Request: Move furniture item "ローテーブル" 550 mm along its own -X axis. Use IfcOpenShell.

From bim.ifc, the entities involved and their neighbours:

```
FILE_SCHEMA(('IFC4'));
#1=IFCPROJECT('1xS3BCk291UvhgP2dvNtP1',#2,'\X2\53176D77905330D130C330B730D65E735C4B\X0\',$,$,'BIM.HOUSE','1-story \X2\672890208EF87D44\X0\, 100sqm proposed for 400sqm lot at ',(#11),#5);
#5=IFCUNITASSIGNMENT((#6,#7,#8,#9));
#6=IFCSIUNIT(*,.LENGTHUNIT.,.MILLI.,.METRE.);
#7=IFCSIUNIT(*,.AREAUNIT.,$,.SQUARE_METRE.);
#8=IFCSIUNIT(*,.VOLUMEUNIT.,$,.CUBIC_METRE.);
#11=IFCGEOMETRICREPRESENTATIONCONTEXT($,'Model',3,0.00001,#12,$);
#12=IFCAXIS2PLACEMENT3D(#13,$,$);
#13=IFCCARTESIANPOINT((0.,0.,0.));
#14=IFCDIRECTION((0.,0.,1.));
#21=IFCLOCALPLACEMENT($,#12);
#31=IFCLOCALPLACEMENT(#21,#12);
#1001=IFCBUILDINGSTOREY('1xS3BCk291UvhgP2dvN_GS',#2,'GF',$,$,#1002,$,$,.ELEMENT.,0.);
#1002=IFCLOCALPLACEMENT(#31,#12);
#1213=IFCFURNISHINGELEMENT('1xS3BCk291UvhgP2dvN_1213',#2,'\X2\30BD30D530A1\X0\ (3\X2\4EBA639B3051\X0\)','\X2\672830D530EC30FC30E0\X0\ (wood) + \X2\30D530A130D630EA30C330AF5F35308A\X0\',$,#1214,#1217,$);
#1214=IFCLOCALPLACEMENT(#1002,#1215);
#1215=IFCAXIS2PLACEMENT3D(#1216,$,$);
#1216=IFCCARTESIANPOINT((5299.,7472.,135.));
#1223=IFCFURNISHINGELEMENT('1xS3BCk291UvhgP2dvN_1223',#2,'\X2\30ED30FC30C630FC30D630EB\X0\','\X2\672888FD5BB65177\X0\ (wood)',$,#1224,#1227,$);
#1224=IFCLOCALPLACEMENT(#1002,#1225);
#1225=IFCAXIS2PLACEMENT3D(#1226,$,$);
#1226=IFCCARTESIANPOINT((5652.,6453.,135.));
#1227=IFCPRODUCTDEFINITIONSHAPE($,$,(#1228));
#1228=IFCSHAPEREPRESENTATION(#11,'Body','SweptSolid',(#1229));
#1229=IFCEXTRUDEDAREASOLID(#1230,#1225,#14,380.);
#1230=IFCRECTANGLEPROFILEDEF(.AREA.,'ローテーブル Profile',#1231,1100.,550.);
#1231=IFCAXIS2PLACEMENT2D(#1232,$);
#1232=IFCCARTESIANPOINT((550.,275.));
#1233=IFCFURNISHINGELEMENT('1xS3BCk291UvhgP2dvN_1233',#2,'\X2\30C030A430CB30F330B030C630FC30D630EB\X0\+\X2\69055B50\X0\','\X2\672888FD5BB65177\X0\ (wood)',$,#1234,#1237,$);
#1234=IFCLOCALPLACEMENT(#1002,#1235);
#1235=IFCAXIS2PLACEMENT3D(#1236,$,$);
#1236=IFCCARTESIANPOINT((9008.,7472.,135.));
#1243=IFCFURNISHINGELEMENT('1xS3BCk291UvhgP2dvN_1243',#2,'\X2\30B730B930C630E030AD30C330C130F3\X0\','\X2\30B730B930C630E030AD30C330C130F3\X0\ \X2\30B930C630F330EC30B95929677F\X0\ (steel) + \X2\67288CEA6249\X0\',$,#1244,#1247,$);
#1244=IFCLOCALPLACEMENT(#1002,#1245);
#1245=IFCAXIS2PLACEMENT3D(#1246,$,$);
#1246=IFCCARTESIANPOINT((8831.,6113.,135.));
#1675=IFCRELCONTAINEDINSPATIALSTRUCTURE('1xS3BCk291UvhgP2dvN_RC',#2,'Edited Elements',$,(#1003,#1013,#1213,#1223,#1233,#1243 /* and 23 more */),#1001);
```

```python
import ifcopenshell
import ifcopenshell.api.geometry
import ifcopenshell.util.placement
import ifcopenshell.util.unit

model = ifcopenshell.open("bim.ifc")
unit_scale = ifcopenshell.util.unit.calculate_unit_scale(model)

item = model.by_guid("1xS3BCk291UvhgP2dvN_1223")
matrix = ifcopenshell.util.placement.get_local_placement(item.ObjectPlacement)
matrix[:3, 3] -= matrix[:3, 0] * 0.55 / unit_scale
ifcopenshell.api.geometry.edit_object_placement(model, product=item, matrix=matrix, is_si=False)

print(ifcopenshell.util.placement.get_local_placement(item.ObjectPlacement).round(3) + 0.0)

model.write("bim_rev.ifc")
```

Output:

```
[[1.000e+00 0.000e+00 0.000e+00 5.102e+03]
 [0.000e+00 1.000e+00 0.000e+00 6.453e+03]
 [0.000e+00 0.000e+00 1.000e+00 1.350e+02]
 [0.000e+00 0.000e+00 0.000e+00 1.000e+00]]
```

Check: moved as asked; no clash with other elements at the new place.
